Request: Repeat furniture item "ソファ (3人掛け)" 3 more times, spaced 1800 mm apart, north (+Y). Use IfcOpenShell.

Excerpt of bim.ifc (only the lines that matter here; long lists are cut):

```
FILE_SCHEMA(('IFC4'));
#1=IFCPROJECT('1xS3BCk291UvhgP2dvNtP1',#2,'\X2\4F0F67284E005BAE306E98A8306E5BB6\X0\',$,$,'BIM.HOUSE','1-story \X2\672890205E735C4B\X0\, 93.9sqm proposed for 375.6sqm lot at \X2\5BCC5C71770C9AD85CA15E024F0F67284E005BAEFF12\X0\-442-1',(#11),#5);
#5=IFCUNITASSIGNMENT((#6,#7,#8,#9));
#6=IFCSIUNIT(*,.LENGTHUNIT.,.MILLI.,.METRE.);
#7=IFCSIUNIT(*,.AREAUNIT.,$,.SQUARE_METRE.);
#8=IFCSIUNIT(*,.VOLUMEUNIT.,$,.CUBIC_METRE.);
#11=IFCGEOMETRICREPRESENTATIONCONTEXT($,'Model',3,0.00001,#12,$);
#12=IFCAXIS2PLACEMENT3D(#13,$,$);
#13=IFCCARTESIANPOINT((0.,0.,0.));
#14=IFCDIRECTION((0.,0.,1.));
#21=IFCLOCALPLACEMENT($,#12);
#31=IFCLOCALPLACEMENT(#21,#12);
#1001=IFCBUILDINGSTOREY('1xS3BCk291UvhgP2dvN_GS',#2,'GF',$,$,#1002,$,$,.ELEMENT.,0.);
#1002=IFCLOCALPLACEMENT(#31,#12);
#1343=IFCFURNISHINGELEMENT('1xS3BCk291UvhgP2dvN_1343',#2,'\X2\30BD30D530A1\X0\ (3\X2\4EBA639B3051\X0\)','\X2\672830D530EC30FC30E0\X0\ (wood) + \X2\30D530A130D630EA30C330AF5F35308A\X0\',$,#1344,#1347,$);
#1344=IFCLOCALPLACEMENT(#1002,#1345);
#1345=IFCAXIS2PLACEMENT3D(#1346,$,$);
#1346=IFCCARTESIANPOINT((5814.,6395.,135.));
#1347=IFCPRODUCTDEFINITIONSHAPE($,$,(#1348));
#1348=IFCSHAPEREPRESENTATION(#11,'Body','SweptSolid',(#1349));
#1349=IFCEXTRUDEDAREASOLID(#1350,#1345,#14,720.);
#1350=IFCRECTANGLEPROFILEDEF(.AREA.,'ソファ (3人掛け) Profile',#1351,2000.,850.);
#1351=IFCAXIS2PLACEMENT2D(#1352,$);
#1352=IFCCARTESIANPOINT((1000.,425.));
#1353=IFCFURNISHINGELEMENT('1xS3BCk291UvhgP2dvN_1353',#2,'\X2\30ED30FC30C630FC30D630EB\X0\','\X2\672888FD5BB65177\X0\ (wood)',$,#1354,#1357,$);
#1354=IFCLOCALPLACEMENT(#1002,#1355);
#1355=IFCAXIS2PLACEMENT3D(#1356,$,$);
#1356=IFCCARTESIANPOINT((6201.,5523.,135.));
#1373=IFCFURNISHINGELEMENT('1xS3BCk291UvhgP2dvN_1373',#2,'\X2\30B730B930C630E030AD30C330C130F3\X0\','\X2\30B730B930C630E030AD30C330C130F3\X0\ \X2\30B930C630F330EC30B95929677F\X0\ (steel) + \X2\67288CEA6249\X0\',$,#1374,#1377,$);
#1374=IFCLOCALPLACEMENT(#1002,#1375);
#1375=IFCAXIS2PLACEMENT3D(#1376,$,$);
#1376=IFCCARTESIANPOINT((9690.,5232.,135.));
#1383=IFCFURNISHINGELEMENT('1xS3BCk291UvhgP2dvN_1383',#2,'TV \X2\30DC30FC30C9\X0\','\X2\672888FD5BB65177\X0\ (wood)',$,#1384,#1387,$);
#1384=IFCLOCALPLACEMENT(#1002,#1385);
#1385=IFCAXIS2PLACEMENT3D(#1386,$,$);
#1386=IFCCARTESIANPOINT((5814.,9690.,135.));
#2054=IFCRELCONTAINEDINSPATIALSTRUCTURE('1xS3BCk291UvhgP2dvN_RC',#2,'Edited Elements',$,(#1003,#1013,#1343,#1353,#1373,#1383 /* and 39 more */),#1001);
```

```python
import numpy as np
import ifcopenshell
import ifcopenshell.api.geometry
import ifcopenshell.api.root
import ifcopenshell.util.element
import ifcopenshell.util.placement
import ifcopenshell.util.unit

model = ifcopenshell.open("bim.ifc")
unit_scale = ifcopenshell.util.unit.calculate_unit_scale(model)


def reuse_history(source, copy):
    """copy_class also copies each property set's owner history, people and application; keep the originals."""
    for rel in copy.IsDefinedBy:
        if rel.is_a("IfcRelDefinesByProperties") and (history := rel.RelatingPropertyDefinition.OwnerHistory):
            rel.RelatingPropertyDefinition.OwnerHistory = source.OwnerHistory
            ifcopenshell.util.element.remove_deep2(model, history)


source = model.by_guid("1xS3BCk291UvhgP2dvN_1343")
base = ifcopenshell.util.placement.get_local_placement(source.ObjectPlacement)
step = np.array([0.0, 1.0, 0.0]) * 1.8 / unit_scale

for i in range(1, 4):
    copy = ifcopenshell.api.root.copy_class(model, product=source)
    copy.Representation = ifcopenshell.util.element.copy_deep(
        model, source.Representation, exclude=["IfcGeometricRepresentationContext", "IfcRepresentationMap"]
    )
    reuse_history(source, copy)
    matrix = base.copy()
    matrix[:3, 3] += i * step
    print("added at", matrix[:3, 3].round(3) + 0.0)
    ifcopenshell.api.geometry.edit_object_placement(model, product=copy, matrix=matrix, is_si=False)

model.write("bim_edited.ifc")
```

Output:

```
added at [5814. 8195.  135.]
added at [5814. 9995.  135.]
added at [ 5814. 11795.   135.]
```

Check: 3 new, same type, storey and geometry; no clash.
